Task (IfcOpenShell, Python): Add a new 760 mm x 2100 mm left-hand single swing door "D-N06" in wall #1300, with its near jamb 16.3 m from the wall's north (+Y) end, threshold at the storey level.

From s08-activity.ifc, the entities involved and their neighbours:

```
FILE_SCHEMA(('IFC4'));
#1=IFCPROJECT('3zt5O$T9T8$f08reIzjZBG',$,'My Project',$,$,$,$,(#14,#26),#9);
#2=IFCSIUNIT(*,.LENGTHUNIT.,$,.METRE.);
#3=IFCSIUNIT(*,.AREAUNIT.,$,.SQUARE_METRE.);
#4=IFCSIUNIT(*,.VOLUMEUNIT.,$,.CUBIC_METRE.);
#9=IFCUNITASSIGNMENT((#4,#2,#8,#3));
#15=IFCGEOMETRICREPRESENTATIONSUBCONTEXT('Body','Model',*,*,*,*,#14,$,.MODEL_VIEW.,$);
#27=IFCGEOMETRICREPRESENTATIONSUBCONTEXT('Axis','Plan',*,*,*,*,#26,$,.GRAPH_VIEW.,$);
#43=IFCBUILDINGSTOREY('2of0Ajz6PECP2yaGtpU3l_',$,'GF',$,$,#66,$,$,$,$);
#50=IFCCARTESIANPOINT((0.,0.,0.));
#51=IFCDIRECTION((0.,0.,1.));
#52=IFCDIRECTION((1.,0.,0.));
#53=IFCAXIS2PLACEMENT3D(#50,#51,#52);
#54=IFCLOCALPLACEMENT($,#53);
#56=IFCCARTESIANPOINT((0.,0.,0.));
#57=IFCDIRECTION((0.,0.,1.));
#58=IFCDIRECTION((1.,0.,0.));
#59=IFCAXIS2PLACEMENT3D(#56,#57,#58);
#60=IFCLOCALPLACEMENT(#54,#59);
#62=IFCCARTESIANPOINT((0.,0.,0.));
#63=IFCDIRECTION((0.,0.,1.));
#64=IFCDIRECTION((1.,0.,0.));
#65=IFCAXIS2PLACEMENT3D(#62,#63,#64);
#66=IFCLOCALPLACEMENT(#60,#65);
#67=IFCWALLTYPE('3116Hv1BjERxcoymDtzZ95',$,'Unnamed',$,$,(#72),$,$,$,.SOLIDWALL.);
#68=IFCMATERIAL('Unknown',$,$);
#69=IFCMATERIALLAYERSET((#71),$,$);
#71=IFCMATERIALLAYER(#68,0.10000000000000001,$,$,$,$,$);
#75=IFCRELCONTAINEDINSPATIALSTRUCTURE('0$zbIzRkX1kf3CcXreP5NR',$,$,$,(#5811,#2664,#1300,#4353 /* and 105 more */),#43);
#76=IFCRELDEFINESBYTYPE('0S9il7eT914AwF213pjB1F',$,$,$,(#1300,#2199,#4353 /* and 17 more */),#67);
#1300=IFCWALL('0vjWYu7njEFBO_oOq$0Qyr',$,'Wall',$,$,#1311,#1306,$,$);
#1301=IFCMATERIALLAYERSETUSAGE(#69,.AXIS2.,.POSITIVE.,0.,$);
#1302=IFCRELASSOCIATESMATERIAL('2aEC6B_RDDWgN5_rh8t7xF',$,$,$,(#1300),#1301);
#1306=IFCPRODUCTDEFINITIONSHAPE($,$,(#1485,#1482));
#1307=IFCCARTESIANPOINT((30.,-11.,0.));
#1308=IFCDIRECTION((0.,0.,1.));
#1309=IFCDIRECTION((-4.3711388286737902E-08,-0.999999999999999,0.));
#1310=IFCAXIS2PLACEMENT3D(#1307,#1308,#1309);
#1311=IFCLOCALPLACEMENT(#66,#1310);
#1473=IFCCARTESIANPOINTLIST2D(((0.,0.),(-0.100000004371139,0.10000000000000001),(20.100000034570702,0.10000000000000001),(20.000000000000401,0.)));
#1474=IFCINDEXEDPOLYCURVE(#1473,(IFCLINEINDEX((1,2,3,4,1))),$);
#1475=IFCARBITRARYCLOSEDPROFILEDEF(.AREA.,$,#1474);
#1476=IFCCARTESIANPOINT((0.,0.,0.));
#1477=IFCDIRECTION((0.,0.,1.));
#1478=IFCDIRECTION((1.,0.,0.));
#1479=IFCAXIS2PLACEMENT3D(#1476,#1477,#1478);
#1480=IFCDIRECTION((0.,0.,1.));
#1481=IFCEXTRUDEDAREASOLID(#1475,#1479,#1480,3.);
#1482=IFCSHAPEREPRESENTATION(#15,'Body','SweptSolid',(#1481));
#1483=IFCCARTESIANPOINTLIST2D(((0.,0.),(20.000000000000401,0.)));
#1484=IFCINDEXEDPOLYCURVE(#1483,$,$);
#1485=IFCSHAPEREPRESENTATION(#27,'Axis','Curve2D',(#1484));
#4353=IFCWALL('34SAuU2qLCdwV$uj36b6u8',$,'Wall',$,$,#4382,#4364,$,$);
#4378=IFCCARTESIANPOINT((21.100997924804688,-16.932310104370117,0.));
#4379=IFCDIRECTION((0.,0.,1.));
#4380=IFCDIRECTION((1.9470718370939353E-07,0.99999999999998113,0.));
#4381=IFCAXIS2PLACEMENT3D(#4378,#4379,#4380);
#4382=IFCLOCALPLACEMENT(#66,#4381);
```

```python
import numpy as np
import ifcopenshell
import ifcopenshell.api.feature
import ifcopenshell.api.geometry
import ifcopenshell.api.root
import ifcopenshell.api.spatial
import ifcopenshell.geom
import ifcopenshell.util.element
import ifcopenshell.util.placement
import ifcopenshell.util.representation
import ifcopenshell.util.shape
import ifcopenshell.util.unit

model = ifcopenshell.open("s08-activity.ifc")
unit_scale = ifcopenshell.util.unit.calculate_unit_scale(model)
settings = ifcopenshell.geom.settings()


def volume(element):
    """Net volume in cubic metres, openings subtracted."""
    shape = ifcopenshell.geom.create_shape(settings, element)
    return ifcopenshell.util.shape.get_volume(shape.geometry)


wall = model.by_id(1300)
storey = ifcopenshell.util.element.get_container(wall, ifc_class="IfcBuildingStorey")
context = ifcopenshell.util.representation.get_context(model, "Model", "Body", "MODEL_VIEW")
before = volume(wall)

width, height, from_end, sill = 0.76, 2.1, 16.3, 0.0  # metres

# The wall runs along its own X axis, and the end named is its -X end.
wall_shape = ifcopenshell.geom.create_shape(settings, wall)
x, y, z = ifcopenshell.util.shape.get_vertices(wall_shape.geometry).T
start = x.min() + from_end
face, thickness = float(y.min()), float(y.max() - y.min())
wall_matrix = ifcopenshell.util.placement.get_local_placement(wall.ObjectPlacement)
level = ifcopenshell.util.placement.get_local_placement(storey.ObjectPlacement)[2, 3]


def in_wall(x, y):
    """Placement at x, y metres in the wall's axes, at sill height."""
    matrix = wall_matrix.copy()
    matrix[:, 3] = wall_matrix @ np.array([x / unit_scale, y / unit_scale, 0.0, 1.0])
    matrix[2, 3] = level + sill / unit_scale
    return matrix


# Opening: a box that overshoots both wall faces by 50 mm.
opening = ifcopenshell.api.root.create_entity(model, ifc_class="IfcOpeningElement", predefined_type="OPENING")
box = ifcopenshell.api.geometry.add_wall_representation(
    model, context=context, length=width, height=height, thickness=thickness + 0.1
)
ifcopenshell.api.geometry.assign_representation(model, product=opening, representation=box)
ifcopenshell.api.geometry.edit_object_placement(model, product=opening, matrix=in_wall(start, face - 0.05), is_si=False)
ifcopenshell.api.feature.add_feature(model, feature=opening, element=wall)

door = ifcopenshell.api.root.create_entity(model, ifc_class="IfcDoor", name="D-N06", predefined_type="DOOR")
door.OverallWidth, door.OverallHeight = width / unit_scale, height / unit_scale
door.OperationType = "SINGLE_SWING_LEFT"
body = ifcopenshell.api.geometry.add_door_representation(
    model,
    context=context,
    overall_width=door.OverallWidth,
    overall_height=door.OverallHeight,
    operation_type="SINGLE_SWING_LEFT",
    lining_properties={"LiningDepth": thickness / unit_scale, "ThresholdDepth": thickness / unit_scale},
)
ifcopenshell.api.geometry.assign_representation(model, product=door, representation=body)
ifcopenshell.api.spatial.assign_container(model, products=[door], relating_structure=storey)
ifcopenshell.api.feature.add_filling(model, opening=opening, element=door)

# The lining spans the wall, so the door starts at the wall face.
ifcopenshell.api.geometry.edit_object_placement(model, product=door, matrix=in_wall(start, face), is_si=False)

after = volume(wall)

print(f"wall volume {before:.3f} -> {after:.3f} m3")

model.write("s08-activity_edited.ifc")
```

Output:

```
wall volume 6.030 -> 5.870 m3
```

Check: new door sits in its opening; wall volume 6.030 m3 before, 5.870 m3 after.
